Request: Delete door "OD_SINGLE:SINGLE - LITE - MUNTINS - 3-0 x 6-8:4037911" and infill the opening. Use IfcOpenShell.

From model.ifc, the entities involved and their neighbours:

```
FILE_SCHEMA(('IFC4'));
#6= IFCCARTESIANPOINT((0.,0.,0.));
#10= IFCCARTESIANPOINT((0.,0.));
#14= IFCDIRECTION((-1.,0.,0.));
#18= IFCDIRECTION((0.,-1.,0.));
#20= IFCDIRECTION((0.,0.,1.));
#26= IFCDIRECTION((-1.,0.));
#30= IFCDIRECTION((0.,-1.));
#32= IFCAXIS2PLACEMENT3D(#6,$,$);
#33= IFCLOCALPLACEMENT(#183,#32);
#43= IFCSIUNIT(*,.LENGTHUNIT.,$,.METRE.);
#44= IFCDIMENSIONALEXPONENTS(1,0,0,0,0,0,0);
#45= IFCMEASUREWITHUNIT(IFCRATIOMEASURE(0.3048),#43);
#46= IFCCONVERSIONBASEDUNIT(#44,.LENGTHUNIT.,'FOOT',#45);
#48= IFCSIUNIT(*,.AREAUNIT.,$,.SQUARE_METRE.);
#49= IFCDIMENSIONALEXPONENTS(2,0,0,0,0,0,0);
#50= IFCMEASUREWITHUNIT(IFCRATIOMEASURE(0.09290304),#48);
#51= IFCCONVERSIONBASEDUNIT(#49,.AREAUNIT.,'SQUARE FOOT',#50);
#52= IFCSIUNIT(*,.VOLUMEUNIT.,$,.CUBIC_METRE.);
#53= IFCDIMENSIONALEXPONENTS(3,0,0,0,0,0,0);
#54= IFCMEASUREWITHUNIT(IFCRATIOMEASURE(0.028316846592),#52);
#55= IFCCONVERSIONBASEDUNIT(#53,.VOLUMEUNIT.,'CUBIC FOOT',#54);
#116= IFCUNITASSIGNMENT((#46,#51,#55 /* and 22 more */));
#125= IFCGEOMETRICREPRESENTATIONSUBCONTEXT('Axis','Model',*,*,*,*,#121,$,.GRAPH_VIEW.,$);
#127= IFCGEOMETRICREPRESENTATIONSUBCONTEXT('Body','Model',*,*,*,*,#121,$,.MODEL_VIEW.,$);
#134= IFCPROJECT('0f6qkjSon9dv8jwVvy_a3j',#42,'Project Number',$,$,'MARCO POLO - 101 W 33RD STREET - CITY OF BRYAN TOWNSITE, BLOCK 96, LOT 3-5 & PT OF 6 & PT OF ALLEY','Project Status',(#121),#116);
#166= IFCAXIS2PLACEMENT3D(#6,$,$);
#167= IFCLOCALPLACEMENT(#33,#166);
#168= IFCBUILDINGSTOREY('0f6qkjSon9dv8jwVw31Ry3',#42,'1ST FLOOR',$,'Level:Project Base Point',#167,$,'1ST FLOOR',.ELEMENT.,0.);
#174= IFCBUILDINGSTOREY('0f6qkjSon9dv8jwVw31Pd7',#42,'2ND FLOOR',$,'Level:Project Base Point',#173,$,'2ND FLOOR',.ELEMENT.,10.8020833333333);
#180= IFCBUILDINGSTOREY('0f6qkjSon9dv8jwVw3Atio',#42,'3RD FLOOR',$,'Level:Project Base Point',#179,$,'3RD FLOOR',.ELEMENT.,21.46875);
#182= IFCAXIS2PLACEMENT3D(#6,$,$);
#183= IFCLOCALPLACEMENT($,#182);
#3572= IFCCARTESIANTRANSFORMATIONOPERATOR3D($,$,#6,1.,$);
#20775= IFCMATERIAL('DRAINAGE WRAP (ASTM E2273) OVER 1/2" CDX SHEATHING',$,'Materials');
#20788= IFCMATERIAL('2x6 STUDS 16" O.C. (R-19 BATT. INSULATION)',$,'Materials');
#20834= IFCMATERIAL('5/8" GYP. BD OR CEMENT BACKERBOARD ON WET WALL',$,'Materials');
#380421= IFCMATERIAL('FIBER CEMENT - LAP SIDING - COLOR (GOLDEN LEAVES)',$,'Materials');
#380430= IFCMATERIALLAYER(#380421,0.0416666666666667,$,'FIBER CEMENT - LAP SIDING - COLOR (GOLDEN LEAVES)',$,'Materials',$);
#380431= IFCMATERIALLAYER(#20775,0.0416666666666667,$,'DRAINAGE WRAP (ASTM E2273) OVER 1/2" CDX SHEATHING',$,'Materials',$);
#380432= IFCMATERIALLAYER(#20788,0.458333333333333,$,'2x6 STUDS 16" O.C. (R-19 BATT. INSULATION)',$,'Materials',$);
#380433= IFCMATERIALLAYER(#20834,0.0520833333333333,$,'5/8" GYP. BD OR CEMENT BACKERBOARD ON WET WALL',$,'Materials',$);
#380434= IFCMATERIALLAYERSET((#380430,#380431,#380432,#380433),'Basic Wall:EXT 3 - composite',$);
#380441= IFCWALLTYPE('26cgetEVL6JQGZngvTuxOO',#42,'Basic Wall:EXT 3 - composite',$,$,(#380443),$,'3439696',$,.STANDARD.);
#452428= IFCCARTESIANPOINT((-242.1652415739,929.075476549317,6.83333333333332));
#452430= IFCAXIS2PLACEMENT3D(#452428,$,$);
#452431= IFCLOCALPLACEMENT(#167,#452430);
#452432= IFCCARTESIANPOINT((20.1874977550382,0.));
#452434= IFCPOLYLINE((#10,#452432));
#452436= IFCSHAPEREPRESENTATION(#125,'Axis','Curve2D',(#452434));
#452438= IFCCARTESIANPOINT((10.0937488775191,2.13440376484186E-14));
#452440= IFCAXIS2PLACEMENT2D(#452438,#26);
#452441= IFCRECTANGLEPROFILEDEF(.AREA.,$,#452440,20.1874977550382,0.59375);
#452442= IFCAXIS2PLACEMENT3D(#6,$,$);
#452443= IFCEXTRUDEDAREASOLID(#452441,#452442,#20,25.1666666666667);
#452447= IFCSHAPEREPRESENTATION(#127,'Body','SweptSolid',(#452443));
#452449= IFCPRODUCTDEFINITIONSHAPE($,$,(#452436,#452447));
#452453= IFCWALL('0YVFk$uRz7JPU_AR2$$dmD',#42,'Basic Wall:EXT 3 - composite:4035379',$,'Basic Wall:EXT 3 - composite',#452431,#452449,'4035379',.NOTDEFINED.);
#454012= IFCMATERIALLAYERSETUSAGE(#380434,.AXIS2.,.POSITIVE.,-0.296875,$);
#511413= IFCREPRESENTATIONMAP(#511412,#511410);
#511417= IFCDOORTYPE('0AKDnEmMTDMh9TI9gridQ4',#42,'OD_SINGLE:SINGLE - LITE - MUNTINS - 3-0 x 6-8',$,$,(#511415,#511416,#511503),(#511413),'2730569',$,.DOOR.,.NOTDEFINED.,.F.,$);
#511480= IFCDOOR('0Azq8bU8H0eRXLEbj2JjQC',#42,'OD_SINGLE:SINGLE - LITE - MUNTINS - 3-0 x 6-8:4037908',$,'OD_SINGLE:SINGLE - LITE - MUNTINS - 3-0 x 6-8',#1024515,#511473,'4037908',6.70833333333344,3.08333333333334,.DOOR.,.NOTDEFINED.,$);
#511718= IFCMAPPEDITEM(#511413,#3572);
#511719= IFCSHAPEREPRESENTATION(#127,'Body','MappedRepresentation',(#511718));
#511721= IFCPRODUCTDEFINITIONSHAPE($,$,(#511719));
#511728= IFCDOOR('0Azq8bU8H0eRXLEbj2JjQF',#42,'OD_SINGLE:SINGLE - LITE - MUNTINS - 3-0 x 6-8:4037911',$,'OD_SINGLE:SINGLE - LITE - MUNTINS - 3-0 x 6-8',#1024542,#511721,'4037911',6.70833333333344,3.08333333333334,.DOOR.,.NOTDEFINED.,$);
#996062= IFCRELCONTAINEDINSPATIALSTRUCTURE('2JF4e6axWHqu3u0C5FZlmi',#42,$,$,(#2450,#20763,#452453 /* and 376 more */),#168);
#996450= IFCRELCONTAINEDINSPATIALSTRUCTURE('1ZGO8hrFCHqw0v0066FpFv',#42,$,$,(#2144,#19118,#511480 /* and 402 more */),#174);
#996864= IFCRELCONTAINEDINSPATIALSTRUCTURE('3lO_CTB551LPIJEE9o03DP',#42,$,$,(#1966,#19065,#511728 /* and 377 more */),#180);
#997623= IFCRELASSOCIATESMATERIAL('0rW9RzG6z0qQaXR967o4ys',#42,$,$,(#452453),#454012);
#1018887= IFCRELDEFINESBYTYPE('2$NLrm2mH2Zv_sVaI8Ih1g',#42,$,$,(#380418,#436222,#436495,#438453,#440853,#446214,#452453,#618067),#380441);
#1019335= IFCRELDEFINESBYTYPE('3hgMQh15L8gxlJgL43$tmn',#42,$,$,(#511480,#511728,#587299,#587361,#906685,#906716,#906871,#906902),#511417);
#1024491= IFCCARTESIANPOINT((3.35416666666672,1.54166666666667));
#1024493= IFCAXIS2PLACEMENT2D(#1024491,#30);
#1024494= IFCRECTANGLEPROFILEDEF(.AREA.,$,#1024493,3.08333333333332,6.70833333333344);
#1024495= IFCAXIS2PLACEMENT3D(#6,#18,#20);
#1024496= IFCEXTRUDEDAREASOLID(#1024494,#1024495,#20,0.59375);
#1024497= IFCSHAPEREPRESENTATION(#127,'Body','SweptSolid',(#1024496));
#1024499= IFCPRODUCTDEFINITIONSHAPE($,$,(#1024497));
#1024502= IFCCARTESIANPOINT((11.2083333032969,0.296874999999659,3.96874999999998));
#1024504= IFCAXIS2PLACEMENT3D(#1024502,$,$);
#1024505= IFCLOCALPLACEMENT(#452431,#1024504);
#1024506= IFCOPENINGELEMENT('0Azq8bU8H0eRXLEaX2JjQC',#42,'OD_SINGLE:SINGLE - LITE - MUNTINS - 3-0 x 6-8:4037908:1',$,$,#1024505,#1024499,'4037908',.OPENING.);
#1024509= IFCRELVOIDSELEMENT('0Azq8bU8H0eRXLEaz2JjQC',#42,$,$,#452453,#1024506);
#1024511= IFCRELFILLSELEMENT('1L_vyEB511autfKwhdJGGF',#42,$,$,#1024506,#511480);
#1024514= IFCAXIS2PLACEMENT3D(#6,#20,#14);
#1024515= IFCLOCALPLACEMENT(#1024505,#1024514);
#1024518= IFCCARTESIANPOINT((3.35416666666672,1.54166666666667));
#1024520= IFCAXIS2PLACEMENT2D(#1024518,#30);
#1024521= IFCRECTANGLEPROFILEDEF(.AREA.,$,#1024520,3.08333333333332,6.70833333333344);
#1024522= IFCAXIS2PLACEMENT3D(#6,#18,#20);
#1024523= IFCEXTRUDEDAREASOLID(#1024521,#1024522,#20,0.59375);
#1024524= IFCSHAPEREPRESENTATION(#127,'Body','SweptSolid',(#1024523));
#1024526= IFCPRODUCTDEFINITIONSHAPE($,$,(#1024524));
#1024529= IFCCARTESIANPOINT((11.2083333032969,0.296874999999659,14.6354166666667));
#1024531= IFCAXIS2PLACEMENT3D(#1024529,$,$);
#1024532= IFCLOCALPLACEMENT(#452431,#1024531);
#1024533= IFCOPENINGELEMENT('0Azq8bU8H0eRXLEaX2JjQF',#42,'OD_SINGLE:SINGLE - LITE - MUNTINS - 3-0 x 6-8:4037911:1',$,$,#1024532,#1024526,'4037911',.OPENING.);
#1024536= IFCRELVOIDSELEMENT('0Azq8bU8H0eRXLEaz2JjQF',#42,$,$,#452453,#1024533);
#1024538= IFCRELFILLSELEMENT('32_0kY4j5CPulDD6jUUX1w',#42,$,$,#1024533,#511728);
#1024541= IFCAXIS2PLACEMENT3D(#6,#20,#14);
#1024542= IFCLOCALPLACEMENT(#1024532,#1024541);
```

```python
import ifcopenshell
import ifcopenshell.api.feature
import ifcopenshell.api.root
import ifcopenshell.geom
import ifcopenshell.util.shape

model = ifcopenshell.open("model.ifc")
settings = ifcopenshell.geom.settings()


def volume(element):
    """Net volume in cubic metres, openings subtracted."""
    shape = ifcopenshell.geom.create_shape(settings, element)
    return ifcopenshell.util.shape.get_volume(shape.geometry)


door = model.by_guid("0Azq8bU8H0eRXLEbj2JjQF")
opening = door.FillsVoids[0].RelatingOpeningElement
wall = opening.VoidsElements[0].RelatingBuildingElement
before = volume(wall)

ifcopenshell.api.root.remove_product(model, product=door)
ifcopenshell.api.feature.remove_feature(model, feature=opening)

after = volume(wall)

print(f"wall volume {before:.3f} -> {after:.3f} m3")

model.write("model-out.ifc")
```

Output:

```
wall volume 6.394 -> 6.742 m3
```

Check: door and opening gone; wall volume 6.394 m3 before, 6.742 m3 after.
